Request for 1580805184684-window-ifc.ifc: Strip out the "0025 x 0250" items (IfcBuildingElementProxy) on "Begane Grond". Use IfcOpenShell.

First a look at what the model holds.

```python
import ifcopenshell
import ifcopenshell.util.element

model = ifcopenshell.open("1580805184684-window-ifc.ifc")
print(model.schema)
storey = next(s for s in model.by_type("IfcBuildingStorey") if s.Name == "Begane Grond")
proxies = [e for e in ifcopenshell.util.element.get_decomposition(storey) if e.is_a("IfcBuildingElementProxy")]
seen = {}
for e in proxies:
    element_type = ifcopenshell.util.element.get_type(e)
    name = element_type.Name if element_type not in (None, e) else None
    seen[name] = seen.get(name, 0) + 1
for name, count in sorted(seen.items(), key=str):
    print(count, "x", name)
```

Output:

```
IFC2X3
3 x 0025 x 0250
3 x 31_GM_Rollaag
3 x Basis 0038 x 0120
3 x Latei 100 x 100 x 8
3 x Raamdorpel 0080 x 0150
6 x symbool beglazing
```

```python
import ifcopenshell
import ifcopenshell.api.root
import ifcopenshell.util.element

model = ifcopenshell.open("1580805184684-window-ifc.ifc")

storey = next(s for s in model.by_type("IfcBuildingStorey") if s.Name == "Begane Grond")
proxies = [e for e in ifcopenshell.util.element.get_decomposition(storey) if e.is_a("IfcBuildingElementProxy")]
targets = [e for e in proxies if (t := ifcopenshell.util.element.get_type(e)) not in (None, e) and t.Name == "0025 x 0250"]

for e in targets:
    ifcopenshell.api.root.remove_product(model, product=e)
print(len(targets), "removed")

model.write("1580805184684-window-ifc_rev.ifc")
```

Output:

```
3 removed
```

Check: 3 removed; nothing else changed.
